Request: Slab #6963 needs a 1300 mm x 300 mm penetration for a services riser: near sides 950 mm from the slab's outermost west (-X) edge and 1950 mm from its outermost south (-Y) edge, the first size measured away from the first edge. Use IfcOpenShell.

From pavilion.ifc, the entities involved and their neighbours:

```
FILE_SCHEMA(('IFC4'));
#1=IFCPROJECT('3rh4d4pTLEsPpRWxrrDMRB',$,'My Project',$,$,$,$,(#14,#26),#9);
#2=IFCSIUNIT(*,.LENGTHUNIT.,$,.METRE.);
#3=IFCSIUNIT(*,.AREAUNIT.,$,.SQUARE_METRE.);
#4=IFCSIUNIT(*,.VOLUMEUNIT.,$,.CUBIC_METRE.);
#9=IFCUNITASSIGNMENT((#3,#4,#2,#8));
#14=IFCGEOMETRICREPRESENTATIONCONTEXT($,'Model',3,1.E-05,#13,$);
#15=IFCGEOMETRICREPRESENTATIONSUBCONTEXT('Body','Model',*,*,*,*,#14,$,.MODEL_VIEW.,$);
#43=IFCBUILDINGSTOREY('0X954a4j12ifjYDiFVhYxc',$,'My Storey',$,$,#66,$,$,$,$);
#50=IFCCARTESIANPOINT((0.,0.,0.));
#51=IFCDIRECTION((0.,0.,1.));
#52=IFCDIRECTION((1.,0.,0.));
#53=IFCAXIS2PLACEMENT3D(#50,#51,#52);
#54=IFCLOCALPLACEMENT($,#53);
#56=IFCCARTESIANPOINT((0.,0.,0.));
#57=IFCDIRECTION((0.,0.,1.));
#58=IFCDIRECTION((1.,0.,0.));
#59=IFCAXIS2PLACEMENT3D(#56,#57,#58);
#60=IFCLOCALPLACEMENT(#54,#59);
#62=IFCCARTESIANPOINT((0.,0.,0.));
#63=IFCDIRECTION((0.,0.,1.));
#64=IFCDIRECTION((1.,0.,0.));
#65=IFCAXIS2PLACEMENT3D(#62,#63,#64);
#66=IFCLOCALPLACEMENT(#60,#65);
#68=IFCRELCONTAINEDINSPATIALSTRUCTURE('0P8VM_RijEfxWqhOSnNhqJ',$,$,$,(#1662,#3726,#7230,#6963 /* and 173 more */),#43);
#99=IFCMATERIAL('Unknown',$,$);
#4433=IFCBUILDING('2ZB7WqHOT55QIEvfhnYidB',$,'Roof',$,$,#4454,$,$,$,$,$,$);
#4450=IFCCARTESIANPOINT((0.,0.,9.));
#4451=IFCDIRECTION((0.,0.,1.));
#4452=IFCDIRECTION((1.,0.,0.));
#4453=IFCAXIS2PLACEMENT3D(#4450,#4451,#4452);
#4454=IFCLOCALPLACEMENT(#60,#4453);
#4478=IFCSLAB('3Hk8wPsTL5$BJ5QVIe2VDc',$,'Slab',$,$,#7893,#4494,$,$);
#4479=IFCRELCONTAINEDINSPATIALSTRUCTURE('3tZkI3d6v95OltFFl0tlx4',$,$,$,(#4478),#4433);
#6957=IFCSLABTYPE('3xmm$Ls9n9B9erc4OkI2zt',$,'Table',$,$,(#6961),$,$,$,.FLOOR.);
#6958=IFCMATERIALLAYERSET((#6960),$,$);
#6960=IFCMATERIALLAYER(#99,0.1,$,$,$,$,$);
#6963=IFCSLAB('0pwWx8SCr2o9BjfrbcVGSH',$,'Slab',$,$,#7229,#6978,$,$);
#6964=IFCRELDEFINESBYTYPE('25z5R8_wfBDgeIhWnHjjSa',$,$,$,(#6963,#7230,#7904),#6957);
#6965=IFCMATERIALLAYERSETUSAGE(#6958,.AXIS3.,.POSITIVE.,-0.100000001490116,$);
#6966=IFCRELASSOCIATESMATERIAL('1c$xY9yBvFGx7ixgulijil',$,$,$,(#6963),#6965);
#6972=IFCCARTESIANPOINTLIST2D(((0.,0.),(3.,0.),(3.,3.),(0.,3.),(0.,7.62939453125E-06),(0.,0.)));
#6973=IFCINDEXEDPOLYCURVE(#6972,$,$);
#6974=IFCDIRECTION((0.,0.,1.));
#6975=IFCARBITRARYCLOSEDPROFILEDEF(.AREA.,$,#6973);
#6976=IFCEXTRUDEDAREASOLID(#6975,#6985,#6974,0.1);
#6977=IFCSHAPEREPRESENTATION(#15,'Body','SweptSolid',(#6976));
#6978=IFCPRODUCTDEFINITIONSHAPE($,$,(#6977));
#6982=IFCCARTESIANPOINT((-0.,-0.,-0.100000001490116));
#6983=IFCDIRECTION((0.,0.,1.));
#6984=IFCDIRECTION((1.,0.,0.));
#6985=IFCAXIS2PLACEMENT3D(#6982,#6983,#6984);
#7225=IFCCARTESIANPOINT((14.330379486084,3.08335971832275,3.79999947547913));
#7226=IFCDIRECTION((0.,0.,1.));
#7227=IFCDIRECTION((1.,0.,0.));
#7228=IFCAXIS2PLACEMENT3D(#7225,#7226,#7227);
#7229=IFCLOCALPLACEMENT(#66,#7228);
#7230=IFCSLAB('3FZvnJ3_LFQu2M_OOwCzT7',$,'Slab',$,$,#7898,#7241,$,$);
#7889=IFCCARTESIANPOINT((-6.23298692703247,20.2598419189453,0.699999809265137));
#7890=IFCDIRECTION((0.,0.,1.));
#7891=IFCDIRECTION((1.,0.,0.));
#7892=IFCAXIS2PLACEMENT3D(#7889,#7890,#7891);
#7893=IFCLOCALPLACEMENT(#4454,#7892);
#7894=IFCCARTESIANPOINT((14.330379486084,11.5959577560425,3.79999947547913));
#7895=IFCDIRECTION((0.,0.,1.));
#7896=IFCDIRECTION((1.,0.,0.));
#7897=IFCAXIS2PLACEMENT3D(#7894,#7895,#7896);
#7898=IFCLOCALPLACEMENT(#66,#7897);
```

```python
import numpy as np
import ifcopenshell
import ifcopenshell.api.feature
import ifcopenshell.api.geometry
import ifcopenshell.api.root
import ifcopenshell.geom
import ifcopenshell.util.placement
import ifcopenshell.util.representation
import ifcopenshell.util.shape
import ifcopenshell.util.unit

model = ifcopenshell.open("pavilion.ifc")
unit_scale = ifcopenshell.util.unit.calculate_unit_scale(model)
settings = ifcopenshell.geom.settings()


def volume(element):
    """Net volume in cubic metres, openings subtracted."""
    shape = ifcopenshell.geom.create_shape(settings, element)
    return ifcopenshell.util.shape.get_volume(shape.geometry)


slab = model.by_guid("0pwWx8SCr2o9BjfrbcVGSH")
before = volume(slab)

# Extent in the slab's own axes, in metres. The edges named are its -X and -Y sides.
slab_shape = ifcopenshell.geom.create_shape(settings, slab)
vertices = ifcopenshell.util.shape.get_vertices(slab_shape.geometry)
x_min, y_min, bottom = vertices.min(axis=0)
top = vertices[:, 2].max()

opening = ifcopenshell.api.root.create_entity(model, ifc_class="IfcOpeningElement", name="Services riser opening", predefined_type="OPENING")
context = ifcopenshell.util.representation.get_context(model, "Model", "Body", "MODEL_VIEW")
width, depth = 1.3, 0.3
outline = [(0.0, 0.0), (width, 0.0), (width, depth), (0.0, depth), (0.0, 0.0)]
# Overshoot both faces by 50 mm so the cut is clean.
shape = ifcopenshell.api.geometry.add_slab_representation(
    model, context=context, depth=top - bottom + 0.1, polyline=outline
)
ifcopenshell.api.geometry.assign_representation(model, product=opening, representation=shape)

matrix = ifcopenshell.util.placement.get_local_placement(slab.ObjectPlacement)
matrix[:, 3] = matrix @ np.append(np.array([x_min + 0.95, y_min + 1.95, bottom - 0.05]) / unit_scale, 1.0)
ifcopenshell.api.geometry.edit_object_placement(model, product=opening, matrix=matrix, is_si=False)
ifcopenshell.api.feature.add_feature(model, feature=opening, element=slab)

after = volume(slab)

print(f"slab volume {before:.3f} -> {after:.3f} m3")

model.write("pavilion_rev.ifc")
```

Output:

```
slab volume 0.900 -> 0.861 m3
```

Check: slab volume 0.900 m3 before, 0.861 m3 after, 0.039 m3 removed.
